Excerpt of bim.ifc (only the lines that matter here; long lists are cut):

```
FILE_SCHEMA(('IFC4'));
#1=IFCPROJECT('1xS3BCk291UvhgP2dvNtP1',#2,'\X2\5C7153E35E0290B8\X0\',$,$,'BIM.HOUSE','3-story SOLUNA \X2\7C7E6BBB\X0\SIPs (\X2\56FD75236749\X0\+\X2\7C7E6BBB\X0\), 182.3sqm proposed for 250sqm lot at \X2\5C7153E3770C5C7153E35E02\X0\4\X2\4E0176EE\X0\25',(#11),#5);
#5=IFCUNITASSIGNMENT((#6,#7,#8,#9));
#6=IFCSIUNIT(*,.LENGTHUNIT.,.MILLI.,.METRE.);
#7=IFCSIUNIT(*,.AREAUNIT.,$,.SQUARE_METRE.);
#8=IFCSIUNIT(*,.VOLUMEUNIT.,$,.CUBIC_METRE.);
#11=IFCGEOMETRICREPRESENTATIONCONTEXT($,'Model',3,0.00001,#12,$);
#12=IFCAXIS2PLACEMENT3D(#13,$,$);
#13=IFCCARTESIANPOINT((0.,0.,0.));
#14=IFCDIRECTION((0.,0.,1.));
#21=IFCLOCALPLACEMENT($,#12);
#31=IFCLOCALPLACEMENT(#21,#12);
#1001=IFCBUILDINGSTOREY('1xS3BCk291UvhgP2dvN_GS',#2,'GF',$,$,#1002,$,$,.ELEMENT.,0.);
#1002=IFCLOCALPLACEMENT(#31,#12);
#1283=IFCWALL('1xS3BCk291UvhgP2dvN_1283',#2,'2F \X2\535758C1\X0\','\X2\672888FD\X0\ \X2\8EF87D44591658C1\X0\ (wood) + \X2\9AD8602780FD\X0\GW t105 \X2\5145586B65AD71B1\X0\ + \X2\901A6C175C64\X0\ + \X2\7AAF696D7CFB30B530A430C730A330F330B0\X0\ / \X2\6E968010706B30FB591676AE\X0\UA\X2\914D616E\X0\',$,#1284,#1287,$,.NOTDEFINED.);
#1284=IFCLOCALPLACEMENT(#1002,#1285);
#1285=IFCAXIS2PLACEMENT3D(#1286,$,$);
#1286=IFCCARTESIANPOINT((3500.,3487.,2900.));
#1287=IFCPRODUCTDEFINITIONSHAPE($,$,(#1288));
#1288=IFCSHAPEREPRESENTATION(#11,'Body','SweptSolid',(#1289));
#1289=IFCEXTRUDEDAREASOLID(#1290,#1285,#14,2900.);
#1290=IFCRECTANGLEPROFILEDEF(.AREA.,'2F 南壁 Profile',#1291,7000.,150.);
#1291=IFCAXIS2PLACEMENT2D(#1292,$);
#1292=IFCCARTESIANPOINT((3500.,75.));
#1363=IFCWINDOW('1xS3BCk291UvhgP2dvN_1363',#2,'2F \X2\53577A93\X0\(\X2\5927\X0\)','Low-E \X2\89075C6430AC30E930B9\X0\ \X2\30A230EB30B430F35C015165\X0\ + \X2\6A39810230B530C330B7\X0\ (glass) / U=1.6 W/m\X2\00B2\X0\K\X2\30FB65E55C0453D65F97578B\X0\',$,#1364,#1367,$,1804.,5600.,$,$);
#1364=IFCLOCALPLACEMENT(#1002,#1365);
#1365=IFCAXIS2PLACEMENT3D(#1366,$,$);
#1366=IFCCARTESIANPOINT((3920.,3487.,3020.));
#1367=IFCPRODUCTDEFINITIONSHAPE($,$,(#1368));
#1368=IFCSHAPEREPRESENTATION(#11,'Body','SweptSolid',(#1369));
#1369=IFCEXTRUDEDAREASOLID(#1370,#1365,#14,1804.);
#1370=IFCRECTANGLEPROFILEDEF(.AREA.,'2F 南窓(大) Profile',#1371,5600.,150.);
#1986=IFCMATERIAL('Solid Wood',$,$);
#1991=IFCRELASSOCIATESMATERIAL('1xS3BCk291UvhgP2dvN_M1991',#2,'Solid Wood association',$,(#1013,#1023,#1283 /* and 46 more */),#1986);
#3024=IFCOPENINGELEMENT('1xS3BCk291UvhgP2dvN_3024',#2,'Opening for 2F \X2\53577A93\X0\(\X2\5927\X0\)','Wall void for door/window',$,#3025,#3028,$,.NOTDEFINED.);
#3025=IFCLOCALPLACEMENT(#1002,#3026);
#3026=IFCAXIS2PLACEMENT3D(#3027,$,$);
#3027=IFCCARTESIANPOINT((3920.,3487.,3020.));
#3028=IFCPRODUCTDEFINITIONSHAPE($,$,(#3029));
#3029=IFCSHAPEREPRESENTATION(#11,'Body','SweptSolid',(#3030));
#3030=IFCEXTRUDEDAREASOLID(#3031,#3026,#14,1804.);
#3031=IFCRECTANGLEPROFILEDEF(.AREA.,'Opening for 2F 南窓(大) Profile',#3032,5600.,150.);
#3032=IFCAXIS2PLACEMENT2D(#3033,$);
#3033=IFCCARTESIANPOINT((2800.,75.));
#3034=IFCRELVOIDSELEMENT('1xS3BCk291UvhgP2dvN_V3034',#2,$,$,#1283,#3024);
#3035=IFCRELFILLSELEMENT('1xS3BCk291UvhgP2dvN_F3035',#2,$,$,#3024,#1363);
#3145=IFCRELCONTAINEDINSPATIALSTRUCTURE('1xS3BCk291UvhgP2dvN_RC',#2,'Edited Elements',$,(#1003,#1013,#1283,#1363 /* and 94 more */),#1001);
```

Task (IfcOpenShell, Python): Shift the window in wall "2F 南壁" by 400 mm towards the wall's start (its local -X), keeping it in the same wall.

```python
import ifcopenshell
import ifcopenshell.api.geometry
import ifcopenshell.util.placement
import ifcopenshell.util.unit

model = ifcopenshell.open("bim.ifc")
unit_scale = ifcopenshell.util.unit.calculate_unit_scale(model)

window = model.by_guid("1xS3BCk291UvhgP2dvN_1363")
opening = window.FillsVoids[0].RelatingOpeningElement
wall = opening.VoidsElements[0].RelatingBuildingElement

wall_matrix = ifcopenshell.util.placement.get_local_placement(wall.ObjectPlacement)
shift = wall_matrix[:3, 0] * -0.4 / unit_scale
before = ifcopenshell.util.placement.get_local_placement(window.ObjectPlacement)[:3, 3].copy()

# The window is not placed relative to its opening, so move both.
for product in (opening, window):
    matrix = ifcopenshell.util.placement.get_local_placement(product.ObjectPlacement)
    matrix[:3, 3] += shift
    ifcopenshell.api.geometry.edit_object_placement(model, product=product, matrix=matrix, is_si=False)

after = ifcopenshell.util.placement.get_local_placement(window.ObjectPlacement)[:3, 3]
print("window moved by", (after - before).round(3) + 0.0)

model.write("bim-out.ifc")
```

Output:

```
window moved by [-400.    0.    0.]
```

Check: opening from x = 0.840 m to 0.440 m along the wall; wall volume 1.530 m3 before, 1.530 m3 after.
